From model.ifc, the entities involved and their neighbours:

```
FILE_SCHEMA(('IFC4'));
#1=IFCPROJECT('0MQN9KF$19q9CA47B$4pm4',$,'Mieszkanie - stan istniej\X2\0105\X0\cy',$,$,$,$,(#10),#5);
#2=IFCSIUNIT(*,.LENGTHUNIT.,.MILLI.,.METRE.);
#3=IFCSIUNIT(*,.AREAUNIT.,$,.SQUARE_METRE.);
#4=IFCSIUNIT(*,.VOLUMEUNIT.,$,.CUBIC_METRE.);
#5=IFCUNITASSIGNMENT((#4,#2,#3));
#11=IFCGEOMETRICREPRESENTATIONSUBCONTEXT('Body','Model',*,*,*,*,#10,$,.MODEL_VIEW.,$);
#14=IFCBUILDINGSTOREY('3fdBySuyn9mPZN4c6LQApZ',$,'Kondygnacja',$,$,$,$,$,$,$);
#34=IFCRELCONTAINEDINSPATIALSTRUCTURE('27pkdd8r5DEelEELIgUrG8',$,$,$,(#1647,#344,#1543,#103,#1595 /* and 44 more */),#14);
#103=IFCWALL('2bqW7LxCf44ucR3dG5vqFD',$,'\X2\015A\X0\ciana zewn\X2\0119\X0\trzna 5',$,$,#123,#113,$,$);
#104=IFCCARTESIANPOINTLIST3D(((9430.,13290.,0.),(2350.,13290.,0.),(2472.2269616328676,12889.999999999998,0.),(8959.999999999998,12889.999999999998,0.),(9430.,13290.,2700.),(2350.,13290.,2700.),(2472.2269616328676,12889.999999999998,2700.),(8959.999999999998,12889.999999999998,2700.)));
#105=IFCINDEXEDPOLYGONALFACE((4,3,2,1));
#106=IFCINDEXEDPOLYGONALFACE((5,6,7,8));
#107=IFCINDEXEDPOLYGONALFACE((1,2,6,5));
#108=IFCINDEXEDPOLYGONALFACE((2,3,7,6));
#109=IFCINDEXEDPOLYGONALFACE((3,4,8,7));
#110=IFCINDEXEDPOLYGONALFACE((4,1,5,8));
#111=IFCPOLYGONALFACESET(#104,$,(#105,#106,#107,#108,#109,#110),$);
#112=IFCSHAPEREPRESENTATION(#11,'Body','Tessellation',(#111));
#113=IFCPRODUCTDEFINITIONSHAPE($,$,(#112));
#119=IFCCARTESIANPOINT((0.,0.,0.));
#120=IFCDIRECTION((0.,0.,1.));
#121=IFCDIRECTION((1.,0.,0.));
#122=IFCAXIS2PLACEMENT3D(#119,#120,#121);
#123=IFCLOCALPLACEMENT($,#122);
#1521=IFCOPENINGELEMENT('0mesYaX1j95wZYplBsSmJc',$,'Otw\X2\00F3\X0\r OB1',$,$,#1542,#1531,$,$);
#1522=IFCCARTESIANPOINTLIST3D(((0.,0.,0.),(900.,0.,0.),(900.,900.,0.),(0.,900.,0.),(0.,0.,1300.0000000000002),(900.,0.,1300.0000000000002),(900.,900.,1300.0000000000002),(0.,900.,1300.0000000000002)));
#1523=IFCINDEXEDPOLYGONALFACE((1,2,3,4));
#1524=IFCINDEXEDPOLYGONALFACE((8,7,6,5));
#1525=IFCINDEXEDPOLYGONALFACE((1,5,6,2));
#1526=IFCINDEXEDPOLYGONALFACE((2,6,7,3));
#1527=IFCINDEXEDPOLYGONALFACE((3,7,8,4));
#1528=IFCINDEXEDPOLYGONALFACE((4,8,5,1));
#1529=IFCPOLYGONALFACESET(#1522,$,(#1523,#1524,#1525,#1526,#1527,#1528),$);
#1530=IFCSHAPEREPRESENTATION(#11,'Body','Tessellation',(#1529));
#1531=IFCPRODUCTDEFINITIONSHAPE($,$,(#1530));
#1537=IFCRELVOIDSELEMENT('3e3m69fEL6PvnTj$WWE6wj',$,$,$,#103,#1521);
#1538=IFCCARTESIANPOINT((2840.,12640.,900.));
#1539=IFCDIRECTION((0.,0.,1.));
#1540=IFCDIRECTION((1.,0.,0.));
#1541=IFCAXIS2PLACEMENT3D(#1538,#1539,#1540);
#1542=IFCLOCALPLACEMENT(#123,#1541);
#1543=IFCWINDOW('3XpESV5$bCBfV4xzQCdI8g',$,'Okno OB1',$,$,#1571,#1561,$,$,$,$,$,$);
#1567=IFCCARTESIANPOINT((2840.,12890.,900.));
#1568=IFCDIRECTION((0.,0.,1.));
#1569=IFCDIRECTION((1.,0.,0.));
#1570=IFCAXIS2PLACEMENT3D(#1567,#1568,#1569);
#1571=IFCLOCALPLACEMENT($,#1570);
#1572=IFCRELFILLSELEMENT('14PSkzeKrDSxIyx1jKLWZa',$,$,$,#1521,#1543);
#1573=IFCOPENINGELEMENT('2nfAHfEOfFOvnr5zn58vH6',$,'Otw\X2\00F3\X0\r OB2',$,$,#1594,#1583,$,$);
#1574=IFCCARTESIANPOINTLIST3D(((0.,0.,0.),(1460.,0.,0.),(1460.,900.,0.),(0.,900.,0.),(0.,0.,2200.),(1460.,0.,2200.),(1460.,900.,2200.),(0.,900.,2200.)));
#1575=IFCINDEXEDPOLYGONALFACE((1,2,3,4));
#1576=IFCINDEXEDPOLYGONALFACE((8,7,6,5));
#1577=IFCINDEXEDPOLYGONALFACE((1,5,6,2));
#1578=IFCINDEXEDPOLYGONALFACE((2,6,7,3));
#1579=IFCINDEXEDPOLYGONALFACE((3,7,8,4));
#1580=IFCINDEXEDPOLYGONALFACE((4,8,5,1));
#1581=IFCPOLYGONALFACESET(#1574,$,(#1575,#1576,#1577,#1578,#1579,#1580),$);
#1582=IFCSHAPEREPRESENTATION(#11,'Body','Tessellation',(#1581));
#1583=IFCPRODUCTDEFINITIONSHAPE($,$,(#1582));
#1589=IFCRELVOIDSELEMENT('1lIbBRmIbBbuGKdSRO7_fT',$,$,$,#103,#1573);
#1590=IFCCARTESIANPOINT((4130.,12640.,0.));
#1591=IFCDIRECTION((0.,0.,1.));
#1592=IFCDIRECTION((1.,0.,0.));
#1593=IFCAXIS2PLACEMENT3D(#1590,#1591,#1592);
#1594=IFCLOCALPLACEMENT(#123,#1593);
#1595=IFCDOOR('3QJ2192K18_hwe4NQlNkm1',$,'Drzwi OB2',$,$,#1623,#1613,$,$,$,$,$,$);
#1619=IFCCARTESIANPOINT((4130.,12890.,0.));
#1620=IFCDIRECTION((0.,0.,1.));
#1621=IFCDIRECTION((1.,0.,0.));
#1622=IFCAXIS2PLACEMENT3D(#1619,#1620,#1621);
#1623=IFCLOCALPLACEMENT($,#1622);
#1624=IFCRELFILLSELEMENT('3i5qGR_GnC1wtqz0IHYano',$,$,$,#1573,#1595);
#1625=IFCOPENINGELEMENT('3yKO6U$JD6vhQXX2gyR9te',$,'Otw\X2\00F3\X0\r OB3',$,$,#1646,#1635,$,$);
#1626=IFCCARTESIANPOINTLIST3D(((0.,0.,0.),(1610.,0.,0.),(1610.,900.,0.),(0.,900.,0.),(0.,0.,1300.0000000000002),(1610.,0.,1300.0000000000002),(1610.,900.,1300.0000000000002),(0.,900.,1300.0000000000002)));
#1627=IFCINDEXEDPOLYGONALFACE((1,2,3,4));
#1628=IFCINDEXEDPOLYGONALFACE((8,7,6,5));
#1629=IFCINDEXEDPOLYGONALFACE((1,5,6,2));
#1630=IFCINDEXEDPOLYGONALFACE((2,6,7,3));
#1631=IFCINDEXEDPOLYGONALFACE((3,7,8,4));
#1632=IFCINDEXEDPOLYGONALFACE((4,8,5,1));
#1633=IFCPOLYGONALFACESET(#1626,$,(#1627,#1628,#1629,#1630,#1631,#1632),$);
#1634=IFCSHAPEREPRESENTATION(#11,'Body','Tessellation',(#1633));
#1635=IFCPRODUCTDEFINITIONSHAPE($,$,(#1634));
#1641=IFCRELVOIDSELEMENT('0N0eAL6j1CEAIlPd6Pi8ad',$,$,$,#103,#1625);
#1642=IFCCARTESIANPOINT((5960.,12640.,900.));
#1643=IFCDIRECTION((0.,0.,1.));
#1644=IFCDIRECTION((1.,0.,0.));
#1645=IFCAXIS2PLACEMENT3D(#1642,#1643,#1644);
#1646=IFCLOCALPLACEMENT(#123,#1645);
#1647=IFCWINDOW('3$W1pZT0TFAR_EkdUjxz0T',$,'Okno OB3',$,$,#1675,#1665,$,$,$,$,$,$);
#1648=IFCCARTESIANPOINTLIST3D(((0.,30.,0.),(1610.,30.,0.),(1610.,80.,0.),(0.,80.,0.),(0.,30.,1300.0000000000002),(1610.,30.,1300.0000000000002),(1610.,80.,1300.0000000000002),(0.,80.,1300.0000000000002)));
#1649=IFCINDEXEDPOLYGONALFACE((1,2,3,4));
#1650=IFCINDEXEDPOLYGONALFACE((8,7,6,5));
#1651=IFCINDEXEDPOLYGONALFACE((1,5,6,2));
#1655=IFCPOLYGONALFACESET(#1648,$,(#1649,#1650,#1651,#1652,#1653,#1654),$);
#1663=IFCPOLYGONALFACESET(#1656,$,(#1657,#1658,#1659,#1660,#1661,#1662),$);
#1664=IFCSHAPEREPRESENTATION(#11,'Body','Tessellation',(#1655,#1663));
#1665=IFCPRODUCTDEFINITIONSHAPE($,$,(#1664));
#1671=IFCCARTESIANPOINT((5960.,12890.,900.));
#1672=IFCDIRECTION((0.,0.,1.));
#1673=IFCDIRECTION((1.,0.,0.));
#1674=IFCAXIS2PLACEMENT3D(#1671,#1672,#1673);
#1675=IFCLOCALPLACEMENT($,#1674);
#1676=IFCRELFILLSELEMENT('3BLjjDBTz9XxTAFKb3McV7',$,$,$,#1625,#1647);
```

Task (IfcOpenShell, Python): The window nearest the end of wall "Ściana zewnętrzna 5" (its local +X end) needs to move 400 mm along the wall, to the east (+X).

```python
import ifcopenshell
import ifcopenshell.api.geometry
import ifcopenshell.util.placement
import ifcopenshell.util.unit

model = ifcopenshell.open("model.ifc")
unit_scale = ifcopenshell.util.unit.calculate_unit_scale(model)

window = model.by_id(1647)
opening = window.FillsVoids[0].RelatingOpeningElement
wall = opening.VoidsElements[0].RelatingBuildingElement

wall_matrix = ifcopenshell.util.placement.get_local_placement(wall.ObjectPlacement)
shift = wall_matrix[:3, 0] * 0.4 / unit_scale
before = ifcopenshell.util.placement.get_local_placement(window.ObjectPlacement)[:3, 3].copy()

# The window is not placed relative to its opening, so move both.
for product in (opening, window):
    matrix = ifcopenshell.util.placement.get_local_placement(product.ObjectPlacement)
    matrix[:3, 3] += shift
    ifcopenshell.api.geometry.edit_object_placement(model, product=product, matrix=matrix, is_si=False)

after = ifcopenshell.util.placement.get_local_placement(window.ObjectPlacement)[:3, 3]
print("window moved by", (after - before).round(3) + 0.0)

model.write("model_v2.ifc")
```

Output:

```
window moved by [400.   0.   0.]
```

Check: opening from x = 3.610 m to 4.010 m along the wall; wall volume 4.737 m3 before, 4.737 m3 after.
